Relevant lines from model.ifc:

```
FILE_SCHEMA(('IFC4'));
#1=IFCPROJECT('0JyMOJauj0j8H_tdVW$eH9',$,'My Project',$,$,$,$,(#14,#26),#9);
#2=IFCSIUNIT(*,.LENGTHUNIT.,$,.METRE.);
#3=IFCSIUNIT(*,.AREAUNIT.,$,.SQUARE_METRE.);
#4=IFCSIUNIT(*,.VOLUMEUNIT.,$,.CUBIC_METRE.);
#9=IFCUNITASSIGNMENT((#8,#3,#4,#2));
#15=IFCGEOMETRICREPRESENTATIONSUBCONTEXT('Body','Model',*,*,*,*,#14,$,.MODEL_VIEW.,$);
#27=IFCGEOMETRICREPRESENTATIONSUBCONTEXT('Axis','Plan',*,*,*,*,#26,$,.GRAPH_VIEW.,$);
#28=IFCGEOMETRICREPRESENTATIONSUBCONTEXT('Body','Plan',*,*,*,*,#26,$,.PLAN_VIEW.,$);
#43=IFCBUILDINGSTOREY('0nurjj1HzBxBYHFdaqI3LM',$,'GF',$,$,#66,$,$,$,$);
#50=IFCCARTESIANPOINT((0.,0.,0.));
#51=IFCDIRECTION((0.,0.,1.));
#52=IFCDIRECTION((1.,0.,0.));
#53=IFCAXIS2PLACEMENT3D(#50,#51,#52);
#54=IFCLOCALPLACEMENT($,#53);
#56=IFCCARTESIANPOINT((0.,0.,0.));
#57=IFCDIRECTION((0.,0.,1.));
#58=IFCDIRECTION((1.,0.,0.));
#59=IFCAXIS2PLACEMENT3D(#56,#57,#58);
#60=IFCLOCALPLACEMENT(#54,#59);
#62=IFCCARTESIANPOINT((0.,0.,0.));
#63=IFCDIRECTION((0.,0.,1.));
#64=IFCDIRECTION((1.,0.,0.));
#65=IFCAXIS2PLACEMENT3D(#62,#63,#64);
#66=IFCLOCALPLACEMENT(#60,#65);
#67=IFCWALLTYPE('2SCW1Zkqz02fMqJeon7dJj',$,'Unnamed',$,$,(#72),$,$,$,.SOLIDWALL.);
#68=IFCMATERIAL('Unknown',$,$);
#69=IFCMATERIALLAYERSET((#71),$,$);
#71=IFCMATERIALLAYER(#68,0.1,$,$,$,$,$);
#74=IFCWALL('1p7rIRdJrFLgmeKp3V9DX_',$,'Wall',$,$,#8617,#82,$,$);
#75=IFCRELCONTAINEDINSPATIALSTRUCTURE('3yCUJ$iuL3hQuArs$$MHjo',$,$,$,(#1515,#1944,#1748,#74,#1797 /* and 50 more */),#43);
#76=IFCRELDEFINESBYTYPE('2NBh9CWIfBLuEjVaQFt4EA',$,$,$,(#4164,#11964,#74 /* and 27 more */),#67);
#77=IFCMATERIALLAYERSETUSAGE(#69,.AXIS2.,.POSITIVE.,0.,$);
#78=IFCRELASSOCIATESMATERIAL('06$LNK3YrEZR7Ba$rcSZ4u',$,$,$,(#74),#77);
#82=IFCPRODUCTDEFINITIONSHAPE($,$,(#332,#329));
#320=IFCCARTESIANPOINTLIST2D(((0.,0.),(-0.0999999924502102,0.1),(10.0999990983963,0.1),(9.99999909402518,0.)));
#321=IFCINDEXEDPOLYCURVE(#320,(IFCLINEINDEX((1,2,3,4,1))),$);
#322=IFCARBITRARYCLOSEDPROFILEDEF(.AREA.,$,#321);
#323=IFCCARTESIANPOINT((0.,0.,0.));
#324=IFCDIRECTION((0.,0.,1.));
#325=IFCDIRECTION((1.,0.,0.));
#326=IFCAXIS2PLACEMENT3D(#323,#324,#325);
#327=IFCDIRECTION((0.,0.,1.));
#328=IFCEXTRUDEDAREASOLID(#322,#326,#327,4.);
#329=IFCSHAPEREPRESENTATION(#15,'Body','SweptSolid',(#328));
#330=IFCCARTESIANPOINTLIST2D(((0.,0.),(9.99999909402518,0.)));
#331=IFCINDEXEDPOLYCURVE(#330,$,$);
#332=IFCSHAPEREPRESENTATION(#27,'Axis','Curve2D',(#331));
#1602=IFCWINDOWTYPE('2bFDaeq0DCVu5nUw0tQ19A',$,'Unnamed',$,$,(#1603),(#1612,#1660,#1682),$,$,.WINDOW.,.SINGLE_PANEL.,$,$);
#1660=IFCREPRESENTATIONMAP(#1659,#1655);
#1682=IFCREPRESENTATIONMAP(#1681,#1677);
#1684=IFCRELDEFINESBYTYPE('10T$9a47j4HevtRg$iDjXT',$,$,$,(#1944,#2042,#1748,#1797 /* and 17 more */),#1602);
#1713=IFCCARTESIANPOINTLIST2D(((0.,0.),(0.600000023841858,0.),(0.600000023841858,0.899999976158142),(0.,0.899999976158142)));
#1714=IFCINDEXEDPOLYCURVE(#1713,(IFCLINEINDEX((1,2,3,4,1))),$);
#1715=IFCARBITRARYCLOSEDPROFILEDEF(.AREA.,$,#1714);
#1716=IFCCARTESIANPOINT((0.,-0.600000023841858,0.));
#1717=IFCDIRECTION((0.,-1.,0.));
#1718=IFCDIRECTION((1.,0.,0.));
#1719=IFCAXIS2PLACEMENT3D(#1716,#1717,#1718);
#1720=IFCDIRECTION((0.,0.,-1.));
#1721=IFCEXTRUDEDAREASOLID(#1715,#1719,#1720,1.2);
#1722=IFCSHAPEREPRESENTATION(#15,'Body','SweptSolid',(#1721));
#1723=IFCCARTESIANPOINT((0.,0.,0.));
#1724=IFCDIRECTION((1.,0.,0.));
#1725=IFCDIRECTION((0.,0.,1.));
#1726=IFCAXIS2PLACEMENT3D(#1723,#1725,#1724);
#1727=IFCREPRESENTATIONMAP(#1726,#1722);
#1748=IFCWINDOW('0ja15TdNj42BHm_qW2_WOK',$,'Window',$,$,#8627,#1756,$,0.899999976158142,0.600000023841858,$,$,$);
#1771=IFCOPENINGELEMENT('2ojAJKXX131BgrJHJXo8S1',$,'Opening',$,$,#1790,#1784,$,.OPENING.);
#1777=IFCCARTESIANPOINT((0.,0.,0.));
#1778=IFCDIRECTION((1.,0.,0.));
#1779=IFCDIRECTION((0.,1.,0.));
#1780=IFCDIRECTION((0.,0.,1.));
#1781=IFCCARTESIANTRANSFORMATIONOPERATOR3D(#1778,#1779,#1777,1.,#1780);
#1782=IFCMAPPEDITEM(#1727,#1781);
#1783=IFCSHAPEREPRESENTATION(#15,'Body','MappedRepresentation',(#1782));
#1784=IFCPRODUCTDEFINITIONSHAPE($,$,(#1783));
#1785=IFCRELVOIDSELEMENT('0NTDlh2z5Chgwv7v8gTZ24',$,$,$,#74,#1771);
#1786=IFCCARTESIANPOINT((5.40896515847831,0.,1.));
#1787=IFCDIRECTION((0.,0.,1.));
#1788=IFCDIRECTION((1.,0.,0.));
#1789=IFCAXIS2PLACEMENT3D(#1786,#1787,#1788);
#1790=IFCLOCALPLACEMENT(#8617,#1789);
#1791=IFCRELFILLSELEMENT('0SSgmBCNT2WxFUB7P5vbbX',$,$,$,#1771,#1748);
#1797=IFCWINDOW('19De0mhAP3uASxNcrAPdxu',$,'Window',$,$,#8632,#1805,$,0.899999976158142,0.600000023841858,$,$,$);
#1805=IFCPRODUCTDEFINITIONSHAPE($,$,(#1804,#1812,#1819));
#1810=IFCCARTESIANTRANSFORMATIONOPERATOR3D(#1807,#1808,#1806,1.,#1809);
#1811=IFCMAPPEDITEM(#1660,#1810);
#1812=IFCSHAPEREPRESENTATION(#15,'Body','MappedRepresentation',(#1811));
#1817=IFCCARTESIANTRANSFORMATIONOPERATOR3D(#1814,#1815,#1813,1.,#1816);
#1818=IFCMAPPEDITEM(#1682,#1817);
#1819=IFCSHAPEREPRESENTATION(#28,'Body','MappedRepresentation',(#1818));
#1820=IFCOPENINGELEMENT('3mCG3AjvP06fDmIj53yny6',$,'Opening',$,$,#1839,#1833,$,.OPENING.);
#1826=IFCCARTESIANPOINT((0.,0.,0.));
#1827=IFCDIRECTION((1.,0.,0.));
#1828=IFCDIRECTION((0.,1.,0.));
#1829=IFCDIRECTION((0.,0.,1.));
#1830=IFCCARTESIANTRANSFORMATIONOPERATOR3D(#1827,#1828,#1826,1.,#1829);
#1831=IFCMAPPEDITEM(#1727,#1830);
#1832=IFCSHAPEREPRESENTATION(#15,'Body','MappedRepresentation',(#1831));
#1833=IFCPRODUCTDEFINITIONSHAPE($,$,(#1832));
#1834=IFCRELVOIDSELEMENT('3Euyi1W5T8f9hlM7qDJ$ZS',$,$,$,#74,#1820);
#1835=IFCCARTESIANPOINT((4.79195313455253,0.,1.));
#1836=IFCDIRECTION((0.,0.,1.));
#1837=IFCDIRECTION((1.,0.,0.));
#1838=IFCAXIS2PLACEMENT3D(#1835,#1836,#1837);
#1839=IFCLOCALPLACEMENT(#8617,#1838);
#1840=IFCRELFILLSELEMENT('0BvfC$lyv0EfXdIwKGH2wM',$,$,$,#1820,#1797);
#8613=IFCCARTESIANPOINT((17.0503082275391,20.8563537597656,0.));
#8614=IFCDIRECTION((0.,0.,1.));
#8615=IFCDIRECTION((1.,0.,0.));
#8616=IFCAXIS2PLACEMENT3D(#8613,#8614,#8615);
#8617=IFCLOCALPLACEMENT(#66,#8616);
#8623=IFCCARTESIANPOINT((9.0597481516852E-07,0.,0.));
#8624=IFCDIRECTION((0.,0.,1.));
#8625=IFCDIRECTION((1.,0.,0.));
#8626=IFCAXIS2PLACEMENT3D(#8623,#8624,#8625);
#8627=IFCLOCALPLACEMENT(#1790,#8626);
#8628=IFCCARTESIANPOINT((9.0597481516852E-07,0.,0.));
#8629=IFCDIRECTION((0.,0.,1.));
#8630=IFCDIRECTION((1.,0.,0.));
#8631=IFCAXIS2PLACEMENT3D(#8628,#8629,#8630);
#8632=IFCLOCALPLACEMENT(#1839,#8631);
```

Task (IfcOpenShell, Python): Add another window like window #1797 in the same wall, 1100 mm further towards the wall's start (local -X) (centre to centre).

```python
import ifcopenshell
import ifcopenshell.api.feature
import ifcopenshell.api.geometry
import ifcopenshell.api.root
import ifcopenshell.geom
import ifcopenshell.util.element
import ifcopenshell.util.placement
import ifcopenshell.util.shape

model = ifcopenshell.open("model.ifc")
settings = ifcopenshell.geom.settings()


def volume(element):
    """Net volume in cubic metres, openings subtracted."""
    shape = ifcopenshell.geom.create_shape(settings, element)
    return ifcopenshell.util.shape.get_volume(shape.geometry)


window = model.by_guid("19De0mhAP3uASxNcrAPdxu")
opening = window.FillsVoids[0].RelatingOpeningElement
wall = opening.VoidsElements[0].RelatingBuildingElement
before = volume(wall)
shift = ifcopenshell.util.placement.get_local_placement(wall.ObjectPlacement)[:3, 0] * -1.1

# copy_class copies the void relationship, type, container and properties, but no geometry.
new_opening = ifcopenshell.api.root.copy_class(model, product=opening)
new_opening.Representation = ifcopenshell.util.element.copy_deep(
    model, opening.Representation, exclude=["IfcGeometricRepresentationContext", "IfcRepresentationMap"]
)
new_window = ifcopenshell.api.root.copy_class(model, product=window)
new_window.Representation = ifcopenshell.util.element.copy_deep(
    model, window.Representation, exclude=["IfcGeometricRepresentationContext", "IfcRepresentationMap"]
)
ifcopenshell.api.feature.add_filling(model, opening=new_opening, element=new_window)

for old, new in ((opening, new_opening), (window, new_window)):
    matrix = ifcopenshell.util.placement.get_local_placement(old.ObjectPlacement)
    matrix[:3, 3] += shift
    ifcopenshell.api.geometry.edit_object_placement(model, product=new, matrix=matrix, is_si=False)

after = volume(wall)

print(f"wall volume {before:.3f} -> {after:.3f} m3")

model.write("model-out.ifc")
```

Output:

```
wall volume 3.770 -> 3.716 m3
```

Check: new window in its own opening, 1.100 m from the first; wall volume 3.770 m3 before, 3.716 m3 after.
